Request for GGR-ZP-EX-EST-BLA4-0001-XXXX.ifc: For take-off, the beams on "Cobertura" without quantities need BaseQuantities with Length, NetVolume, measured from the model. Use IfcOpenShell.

First a look at what the model holds.

```python
import ifcopenshell
import ifcopenshell.util.element
import ifcopenshell.util.unit

model = ifcopenshell.open("GGR-ZP-EX-EST-BLA4-0001-XXXX.ifc")
print(model.schema)
for unit_type in ("LENGTHUNIT", "AREAUNIT", "VOLUMEUNIT"):
    print(unit_type, ifcopenshell.util.unit.calculate_unit_scale(model, unit_type))
storey = next(s for s in model.by_type("IfcBuildingStorey") if s.Name == "Cobertura")
beams = [e for e in ifcopenshell.util.element.get_decomposition(storey) if e.is_a("IfcBeam")]
for e in sorted(beams, key=lambda e: e.id()):
    print(e.id(), e.is_a(), e.Name, list(ifcopenshell.util.element.get_psets(e, qtos_only=True)), sep=" | ")
```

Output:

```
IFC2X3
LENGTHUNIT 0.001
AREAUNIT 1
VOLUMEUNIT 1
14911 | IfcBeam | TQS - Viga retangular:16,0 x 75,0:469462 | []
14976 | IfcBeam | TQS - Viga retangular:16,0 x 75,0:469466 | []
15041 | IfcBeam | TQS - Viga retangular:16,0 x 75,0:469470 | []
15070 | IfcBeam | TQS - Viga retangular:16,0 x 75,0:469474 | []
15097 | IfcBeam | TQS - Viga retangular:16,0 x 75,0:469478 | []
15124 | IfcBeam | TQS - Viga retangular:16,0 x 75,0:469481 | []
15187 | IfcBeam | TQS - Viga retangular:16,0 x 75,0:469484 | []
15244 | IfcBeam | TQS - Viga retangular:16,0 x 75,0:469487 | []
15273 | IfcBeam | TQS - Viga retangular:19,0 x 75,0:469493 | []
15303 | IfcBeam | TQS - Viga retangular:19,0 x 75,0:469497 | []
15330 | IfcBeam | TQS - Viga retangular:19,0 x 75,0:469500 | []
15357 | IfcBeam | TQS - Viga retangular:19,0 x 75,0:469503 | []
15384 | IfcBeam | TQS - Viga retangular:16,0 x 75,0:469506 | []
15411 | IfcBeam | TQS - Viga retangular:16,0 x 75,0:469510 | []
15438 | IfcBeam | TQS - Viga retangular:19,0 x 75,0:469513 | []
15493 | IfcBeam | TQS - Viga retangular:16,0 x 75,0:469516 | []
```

```python
import ifcopenshell
import ifcopenshell.api.pset
import ifcopenshell.geom
import ifcopenshell.util.element
import ifcopenshell.util.shape
import ifcopenshell.util.unit

model = ifcopenshell.open("GGR-ZP-EX-EST-BLA4-0001-XXXX.ifc")
unit_scale = ifcopenshell.util.unit.calculate_unit_scale(model)
volume_scale = ifcopenshell.util.unit.calculate_unit_scale(model, "VOLUMEUNIT")
settings = ifcopenshell.geom.settings()

storey = next(s for s in model.by_type("IfcBuildingStorey") if s.Name == "Cobertura")
beams = [e for e in ifcopenshell.util.element.get_decomposition(storey) if e.is_a("IfcBeam")]

for e in sorted(beams, key=lambda e: e.id()):
    if ifcopenshell.util.element.get_psets(e, qtos_only=True, should_inherit=False):
        continue
    # Geometry comes back in metres, in the element's own axes.
    shape = ifcopenshell.geom.create_shape(settings, e)
    values = {
        "Length": ifcopenshell.util.shape.get_max_xyz(shape.geometry) / unit_scale,
        "NetVolume": ifcopenshell.util.shape.get_volume(shape.geometry) / volume_scale,
    }
    qto = ifcopenshell.api.pset.add_qto(model, product=e, name="BaseQuantities")
    ifcopenshell.api.pset.edit_qto(model, qto=qto, properties=values)
    print(e.id(), {k: round(v, 3) for k, v in values.items()})

model.write("GGR-ZP-EX-EST-BLA4-0001-XXXX_rev.ifc")
```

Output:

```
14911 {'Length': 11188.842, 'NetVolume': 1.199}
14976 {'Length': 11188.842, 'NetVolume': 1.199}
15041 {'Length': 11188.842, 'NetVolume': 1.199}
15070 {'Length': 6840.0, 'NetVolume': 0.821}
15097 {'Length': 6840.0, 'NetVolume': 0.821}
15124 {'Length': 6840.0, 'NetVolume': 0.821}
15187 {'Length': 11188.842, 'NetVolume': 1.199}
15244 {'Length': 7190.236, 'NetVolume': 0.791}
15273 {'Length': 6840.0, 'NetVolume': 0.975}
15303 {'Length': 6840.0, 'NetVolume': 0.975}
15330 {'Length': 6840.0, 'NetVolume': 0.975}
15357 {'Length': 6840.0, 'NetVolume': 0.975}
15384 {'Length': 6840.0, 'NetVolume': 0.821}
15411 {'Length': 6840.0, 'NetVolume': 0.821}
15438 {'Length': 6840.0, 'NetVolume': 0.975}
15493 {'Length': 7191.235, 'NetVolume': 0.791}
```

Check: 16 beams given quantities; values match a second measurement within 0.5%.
